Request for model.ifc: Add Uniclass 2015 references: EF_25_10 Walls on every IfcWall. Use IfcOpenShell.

First a look at what the model holds.

```python
import ifcopenshell

model = ifcopenshell.open("model.ifc")
print(model.schema)
print("classifications:", [c.Name for c in model.by_type("IfcClassification")])
for ifc_class in ("IfcDoor", "IfcRoof", "IfcStair", "IfcWall", "IfcWindow"):
    print(ifc_class, len(model.by_type(ifc_class)))
```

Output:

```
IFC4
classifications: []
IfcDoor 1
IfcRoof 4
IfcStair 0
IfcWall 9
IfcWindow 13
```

```python
import ifcopenshell
import ifcopenshell.api.classification

model = ifcopenshell.open("model.ifc")

system = ifcopenshell.api.classification.add_classification(model, classification="Uniclass 2015")

codes = {
    "IfcWall": ("EF_25_10", "Walls"),
}
for ifc_class, (code, name) in codes.items():
    products = model.by_type(ifc_class)
    ifcopenshell.api.classification.add_reference(
        model, products=products, classification=system, identification=code, name=name
    )
    print(code, len(products))

model.write("model_updated.ifc")
```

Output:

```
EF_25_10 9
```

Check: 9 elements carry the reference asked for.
